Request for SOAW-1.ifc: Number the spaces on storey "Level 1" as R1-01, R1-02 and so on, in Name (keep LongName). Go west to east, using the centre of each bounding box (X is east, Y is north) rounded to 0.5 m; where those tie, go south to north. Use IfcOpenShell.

First a look at what the model holds.

```python
import ifcopenshell
import ifcopenshell.util.element
import ifcopenshell.util.placement

model = ifcopenshell.open("SOAW-1.ifc")
print(model.schema)
storey = next(s for s in model.by_type("IfcBuildingStorey") if s.Name == "Level 1")
spaces = [e for e in ifcopenshell.util.element.get_decomposition(storey) if e.is_a("IfcSpace")]
for e in sorted(spaces, key=lambda e: e.id()):
    origin = ifcopenshell.util.placement.get_local_placement(e.ObjectPlacement)[:3, 3]
    print(e.id(), e.Name, e.LongName, origin.round(2) + 0.0, sep=" | ")
```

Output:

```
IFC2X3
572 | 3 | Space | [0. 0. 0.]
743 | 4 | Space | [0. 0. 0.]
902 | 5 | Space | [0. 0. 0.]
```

```python
import ifcopenshell
import ifcopenshell.geom
import ifcopenshell.util.element
import ifcopenshell.util.shape

model = ifcopenshell.open("SOAW-1.ifc")
settings = ifcopenshell.geom.settings()
settings.set("use-world-coords", True)


def centre(element):
    shape = ifcopenshell.geom.create_shape(settings, element)
    return ifcopenshell.util.shape.get_bbox_centroid(shape.geometry)


storey = next(s for s in model.by_type("IfcBuildingStorey") if s.Name == "Level 1")
spaces = [e for e in ifcopenshell.util.element.get_decomposition(storey) if e.is_a("IfcSpace")]

# Insertion points can sit at a corner or the storey origin, so sort by the geometry (in metres).
centres = {e: centre(e) for e in spaces}
spaces.sort(key=lambda e: (round(centres[e][0] / 0.5), centres[e][1]))

for i, e in enumerate(spaces, start=1):
    number = f"R1-{i:02d}"
    e.Name = number
    print(e.id(), number)

model.write("SOAW-1_updated.ifc")
```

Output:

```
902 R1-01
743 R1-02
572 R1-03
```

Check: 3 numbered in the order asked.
